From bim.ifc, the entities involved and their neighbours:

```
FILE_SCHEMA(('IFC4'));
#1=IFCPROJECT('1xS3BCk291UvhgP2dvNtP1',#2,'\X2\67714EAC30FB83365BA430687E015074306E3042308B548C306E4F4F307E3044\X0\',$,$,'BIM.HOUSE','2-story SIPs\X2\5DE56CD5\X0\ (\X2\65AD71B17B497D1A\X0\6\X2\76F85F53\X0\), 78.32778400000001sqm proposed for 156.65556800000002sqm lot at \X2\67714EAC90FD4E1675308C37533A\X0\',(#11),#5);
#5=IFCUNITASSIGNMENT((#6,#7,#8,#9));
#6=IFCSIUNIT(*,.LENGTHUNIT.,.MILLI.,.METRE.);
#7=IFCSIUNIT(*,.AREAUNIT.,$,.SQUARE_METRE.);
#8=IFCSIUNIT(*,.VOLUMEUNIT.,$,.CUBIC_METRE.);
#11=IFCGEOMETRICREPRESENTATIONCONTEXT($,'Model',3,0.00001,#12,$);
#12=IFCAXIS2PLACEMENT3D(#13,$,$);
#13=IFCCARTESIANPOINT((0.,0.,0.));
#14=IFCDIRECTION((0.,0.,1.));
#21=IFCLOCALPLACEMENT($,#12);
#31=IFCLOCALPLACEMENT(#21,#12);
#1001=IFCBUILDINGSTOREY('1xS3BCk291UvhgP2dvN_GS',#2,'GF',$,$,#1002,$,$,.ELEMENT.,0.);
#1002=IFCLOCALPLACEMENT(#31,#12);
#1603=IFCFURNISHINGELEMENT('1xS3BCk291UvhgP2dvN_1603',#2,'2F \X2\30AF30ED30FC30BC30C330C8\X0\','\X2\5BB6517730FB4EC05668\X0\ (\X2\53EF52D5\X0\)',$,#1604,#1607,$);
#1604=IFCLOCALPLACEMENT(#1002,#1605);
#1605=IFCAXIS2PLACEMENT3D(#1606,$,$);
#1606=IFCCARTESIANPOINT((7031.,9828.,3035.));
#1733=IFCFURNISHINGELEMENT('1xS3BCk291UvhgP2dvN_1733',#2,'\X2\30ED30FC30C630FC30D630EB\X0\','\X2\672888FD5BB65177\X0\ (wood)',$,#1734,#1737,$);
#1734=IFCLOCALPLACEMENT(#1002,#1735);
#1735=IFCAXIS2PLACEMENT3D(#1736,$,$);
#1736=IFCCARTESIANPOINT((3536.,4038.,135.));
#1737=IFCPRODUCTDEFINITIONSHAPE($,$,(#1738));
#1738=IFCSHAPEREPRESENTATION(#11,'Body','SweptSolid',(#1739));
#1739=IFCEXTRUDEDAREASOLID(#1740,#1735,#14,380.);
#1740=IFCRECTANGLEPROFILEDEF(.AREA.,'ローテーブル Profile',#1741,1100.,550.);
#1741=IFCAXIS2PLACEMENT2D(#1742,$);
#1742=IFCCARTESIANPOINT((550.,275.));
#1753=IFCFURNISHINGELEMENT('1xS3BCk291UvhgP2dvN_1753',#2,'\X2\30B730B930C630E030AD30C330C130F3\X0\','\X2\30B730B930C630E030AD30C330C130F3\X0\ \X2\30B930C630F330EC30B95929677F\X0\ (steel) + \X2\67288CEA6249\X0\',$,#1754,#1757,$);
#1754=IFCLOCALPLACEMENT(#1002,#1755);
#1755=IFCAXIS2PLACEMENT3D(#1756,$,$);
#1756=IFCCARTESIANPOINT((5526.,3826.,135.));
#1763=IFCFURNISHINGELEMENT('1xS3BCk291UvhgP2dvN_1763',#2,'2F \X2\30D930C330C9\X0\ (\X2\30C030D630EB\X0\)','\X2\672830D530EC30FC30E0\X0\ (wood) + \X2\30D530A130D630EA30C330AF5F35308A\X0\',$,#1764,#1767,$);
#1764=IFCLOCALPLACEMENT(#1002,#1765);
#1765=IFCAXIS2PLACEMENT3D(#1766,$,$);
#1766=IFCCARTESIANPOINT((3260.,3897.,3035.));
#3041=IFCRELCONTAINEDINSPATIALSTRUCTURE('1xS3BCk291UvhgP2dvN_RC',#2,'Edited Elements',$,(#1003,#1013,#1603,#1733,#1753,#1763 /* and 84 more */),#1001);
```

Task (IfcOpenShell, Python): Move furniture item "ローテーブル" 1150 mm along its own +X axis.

```python
import ifcopenshell
import ifcopenshell.api.geometry
import ifcopenshell.util.placement
import ifcopenshell.util.unit

model = ifcopenshell.open("bim.ifc")
unit_scale = ifcopenshell.util.unit.calculate_unit_scale(model)

item = model.by_guid("1xS3BCk291UvhgP2dvN_1733")
matrix = ifcopenshell.util.placement.get_local_placement(item.ObjectPlacement)
matrix[:3, 3] += matrix[:3, 0] * 1.15 / unit_scale
ifcopenshell.api.geometry.edit_object_placement(model, product=item, matrix=matrix, is_si=False)

print(ifcopenshell.util.placement.get_local_placement(item.ObjectPlacement).round(3) + 0.0)

model.write("bim_edited.ifc")
```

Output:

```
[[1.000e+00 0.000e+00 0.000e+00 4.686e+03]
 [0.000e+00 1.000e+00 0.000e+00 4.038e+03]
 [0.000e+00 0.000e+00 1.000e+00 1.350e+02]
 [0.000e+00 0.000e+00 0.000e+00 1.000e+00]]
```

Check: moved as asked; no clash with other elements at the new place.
